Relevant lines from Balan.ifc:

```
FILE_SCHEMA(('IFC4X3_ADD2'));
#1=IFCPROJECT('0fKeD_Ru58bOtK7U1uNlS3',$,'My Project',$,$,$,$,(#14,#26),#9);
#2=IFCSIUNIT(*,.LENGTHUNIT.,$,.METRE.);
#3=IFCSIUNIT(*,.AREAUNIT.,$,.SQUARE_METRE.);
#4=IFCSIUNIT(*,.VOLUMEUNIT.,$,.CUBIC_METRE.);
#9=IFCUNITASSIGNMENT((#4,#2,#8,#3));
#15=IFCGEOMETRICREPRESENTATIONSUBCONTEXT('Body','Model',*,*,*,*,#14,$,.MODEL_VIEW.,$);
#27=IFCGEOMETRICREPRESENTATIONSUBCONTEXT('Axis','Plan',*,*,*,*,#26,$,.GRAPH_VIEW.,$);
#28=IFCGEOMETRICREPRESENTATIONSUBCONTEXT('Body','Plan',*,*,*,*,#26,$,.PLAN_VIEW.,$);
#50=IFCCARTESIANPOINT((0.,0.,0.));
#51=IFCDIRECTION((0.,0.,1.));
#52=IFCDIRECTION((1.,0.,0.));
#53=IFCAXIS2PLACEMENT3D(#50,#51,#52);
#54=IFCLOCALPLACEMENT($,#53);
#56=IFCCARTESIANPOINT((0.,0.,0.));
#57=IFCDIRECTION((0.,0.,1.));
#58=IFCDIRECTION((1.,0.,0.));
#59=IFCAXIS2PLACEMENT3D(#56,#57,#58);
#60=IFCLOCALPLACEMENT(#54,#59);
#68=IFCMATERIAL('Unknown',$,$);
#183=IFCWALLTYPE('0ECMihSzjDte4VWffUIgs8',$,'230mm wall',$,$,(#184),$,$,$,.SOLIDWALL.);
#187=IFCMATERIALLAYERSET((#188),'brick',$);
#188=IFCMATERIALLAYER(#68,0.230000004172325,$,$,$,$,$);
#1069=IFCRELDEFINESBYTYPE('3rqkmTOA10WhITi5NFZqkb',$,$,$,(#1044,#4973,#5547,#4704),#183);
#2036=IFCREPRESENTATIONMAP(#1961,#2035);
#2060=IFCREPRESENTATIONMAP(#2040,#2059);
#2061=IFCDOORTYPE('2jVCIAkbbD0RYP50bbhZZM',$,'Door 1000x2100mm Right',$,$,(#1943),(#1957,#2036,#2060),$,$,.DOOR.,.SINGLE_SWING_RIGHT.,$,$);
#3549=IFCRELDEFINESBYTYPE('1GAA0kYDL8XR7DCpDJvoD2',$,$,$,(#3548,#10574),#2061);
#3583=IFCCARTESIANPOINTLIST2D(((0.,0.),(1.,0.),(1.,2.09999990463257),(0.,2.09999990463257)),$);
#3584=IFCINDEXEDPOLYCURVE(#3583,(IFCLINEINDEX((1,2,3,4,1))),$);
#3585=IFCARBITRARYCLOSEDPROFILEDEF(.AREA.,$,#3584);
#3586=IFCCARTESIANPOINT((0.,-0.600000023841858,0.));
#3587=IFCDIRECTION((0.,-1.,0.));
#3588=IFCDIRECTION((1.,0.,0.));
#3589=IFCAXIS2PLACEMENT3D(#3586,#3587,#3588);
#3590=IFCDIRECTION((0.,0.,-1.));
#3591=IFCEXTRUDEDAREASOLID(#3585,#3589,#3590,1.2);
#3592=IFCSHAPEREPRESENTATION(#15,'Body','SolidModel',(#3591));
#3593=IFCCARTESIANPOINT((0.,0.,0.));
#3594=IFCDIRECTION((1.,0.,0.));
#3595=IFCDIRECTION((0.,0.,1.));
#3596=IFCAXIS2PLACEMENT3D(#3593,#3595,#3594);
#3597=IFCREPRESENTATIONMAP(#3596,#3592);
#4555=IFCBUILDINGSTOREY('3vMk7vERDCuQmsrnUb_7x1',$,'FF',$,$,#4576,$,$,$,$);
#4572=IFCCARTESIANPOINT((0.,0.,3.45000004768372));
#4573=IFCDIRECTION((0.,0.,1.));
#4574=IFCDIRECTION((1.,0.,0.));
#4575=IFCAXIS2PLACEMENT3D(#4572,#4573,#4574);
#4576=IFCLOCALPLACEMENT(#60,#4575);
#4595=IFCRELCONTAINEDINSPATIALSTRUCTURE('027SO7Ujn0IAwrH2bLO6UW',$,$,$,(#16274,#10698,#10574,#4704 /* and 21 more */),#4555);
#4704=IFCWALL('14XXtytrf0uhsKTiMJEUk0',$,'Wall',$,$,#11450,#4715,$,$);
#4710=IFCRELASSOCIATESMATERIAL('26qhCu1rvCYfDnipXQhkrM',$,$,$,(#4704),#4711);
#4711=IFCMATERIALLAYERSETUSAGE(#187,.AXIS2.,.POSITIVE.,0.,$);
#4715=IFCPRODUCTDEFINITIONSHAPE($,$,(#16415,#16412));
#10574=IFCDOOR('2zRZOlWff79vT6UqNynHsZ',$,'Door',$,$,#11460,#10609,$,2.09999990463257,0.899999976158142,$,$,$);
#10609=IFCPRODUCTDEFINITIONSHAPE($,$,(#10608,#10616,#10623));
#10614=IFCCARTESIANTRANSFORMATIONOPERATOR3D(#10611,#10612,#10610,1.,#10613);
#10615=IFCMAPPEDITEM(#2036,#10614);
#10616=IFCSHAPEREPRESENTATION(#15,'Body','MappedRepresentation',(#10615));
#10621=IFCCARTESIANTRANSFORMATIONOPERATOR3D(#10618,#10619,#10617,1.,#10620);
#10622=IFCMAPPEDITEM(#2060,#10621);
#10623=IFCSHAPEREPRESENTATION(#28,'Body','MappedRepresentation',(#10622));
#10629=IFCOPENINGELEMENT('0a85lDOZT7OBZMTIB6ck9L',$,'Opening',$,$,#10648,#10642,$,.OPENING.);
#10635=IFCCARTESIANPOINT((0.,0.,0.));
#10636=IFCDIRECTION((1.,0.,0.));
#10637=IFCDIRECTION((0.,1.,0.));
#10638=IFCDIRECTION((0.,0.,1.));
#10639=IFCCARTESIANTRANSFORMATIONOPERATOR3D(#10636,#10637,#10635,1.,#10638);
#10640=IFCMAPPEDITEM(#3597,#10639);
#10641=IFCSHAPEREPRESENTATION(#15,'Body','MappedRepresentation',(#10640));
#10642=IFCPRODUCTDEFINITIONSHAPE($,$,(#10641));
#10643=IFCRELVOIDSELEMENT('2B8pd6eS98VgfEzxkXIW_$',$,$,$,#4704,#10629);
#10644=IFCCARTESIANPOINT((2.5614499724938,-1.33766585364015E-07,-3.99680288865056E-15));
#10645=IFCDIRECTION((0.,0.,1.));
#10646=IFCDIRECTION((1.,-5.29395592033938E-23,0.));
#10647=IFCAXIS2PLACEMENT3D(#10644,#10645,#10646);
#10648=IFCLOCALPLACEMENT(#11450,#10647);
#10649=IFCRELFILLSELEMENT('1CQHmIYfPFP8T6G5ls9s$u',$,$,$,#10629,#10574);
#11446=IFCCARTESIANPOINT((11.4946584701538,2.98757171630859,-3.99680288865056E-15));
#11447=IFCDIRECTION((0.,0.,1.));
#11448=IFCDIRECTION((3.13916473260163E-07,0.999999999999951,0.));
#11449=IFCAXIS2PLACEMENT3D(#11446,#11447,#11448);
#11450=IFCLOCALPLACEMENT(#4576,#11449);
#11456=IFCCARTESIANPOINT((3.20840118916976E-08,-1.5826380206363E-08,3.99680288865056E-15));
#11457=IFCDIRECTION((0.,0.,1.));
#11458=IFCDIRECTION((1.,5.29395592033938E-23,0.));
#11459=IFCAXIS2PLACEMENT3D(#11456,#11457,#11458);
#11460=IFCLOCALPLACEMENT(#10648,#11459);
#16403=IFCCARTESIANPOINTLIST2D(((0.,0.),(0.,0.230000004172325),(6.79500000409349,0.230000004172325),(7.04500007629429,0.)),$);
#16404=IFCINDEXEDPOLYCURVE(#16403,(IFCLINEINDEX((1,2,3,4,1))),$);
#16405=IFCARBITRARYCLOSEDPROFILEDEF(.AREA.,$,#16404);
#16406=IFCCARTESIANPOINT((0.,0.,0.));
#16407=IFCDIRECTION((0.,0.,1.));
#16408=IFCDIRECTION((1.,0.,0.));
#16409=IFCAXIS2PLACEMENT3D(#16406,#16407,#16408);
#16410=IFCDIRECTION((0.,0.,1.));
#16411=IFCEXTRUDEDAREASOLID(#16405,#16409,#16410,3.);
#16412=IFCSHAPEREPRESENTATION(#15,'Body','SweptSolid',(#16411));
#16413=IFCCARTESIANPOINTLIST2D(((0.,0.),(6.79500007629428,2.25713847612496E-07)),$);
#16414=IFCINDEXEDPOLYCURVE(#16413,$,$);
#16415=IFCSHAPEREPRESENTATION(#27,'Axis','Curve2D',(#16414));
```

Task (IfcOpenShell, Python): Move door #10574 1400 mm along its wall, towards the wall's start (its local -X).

```python
import ifcopenshell
import ifcopenshell.api.geometry
import ifcopenshell.util.placement

model = ifcopenshell.open("Balan.ifc")

door = model.by_guid("2zRZOlWff79vT6UqNynHsZ")
opening = door.FillsVoids[0].RelatingOpeningElement
wall = opening.VoidsElements[0].RelatingBuildingElement

wall_matrix = ifcopenshell.util.placement.get_local_placement(wall.ObjectPlacement)
shift = wall_matrix[:3, 0] * -1.4
before = ifcopenshell.util.placement.get_local_placement(door.ObjectPlacement)[:3, 3].copy()

# The door is placed relative to its opening, so it follows when the opening moves.
matrix = ifcopenshell.util.placement.get_local_placement(opening.ObjectPlacement)
matrix[:3, 3] += shift
ifcopenshell.api.geometry.edit_object_placement(
    model, product=opening, matrix=matrix, is_si=False, should_transform_children=True
)

after = ifcopenshell.util.placement.get_local_placement(door.ObjectPlacement)[:3, 3]
print("door moved by", (after - before).round(3) + 0.0)

model.write("Balan-out.ifc")
```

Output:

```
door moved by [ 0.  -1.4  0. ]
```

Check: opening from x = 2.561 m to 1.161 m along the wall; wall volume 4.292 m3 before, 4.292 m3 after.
